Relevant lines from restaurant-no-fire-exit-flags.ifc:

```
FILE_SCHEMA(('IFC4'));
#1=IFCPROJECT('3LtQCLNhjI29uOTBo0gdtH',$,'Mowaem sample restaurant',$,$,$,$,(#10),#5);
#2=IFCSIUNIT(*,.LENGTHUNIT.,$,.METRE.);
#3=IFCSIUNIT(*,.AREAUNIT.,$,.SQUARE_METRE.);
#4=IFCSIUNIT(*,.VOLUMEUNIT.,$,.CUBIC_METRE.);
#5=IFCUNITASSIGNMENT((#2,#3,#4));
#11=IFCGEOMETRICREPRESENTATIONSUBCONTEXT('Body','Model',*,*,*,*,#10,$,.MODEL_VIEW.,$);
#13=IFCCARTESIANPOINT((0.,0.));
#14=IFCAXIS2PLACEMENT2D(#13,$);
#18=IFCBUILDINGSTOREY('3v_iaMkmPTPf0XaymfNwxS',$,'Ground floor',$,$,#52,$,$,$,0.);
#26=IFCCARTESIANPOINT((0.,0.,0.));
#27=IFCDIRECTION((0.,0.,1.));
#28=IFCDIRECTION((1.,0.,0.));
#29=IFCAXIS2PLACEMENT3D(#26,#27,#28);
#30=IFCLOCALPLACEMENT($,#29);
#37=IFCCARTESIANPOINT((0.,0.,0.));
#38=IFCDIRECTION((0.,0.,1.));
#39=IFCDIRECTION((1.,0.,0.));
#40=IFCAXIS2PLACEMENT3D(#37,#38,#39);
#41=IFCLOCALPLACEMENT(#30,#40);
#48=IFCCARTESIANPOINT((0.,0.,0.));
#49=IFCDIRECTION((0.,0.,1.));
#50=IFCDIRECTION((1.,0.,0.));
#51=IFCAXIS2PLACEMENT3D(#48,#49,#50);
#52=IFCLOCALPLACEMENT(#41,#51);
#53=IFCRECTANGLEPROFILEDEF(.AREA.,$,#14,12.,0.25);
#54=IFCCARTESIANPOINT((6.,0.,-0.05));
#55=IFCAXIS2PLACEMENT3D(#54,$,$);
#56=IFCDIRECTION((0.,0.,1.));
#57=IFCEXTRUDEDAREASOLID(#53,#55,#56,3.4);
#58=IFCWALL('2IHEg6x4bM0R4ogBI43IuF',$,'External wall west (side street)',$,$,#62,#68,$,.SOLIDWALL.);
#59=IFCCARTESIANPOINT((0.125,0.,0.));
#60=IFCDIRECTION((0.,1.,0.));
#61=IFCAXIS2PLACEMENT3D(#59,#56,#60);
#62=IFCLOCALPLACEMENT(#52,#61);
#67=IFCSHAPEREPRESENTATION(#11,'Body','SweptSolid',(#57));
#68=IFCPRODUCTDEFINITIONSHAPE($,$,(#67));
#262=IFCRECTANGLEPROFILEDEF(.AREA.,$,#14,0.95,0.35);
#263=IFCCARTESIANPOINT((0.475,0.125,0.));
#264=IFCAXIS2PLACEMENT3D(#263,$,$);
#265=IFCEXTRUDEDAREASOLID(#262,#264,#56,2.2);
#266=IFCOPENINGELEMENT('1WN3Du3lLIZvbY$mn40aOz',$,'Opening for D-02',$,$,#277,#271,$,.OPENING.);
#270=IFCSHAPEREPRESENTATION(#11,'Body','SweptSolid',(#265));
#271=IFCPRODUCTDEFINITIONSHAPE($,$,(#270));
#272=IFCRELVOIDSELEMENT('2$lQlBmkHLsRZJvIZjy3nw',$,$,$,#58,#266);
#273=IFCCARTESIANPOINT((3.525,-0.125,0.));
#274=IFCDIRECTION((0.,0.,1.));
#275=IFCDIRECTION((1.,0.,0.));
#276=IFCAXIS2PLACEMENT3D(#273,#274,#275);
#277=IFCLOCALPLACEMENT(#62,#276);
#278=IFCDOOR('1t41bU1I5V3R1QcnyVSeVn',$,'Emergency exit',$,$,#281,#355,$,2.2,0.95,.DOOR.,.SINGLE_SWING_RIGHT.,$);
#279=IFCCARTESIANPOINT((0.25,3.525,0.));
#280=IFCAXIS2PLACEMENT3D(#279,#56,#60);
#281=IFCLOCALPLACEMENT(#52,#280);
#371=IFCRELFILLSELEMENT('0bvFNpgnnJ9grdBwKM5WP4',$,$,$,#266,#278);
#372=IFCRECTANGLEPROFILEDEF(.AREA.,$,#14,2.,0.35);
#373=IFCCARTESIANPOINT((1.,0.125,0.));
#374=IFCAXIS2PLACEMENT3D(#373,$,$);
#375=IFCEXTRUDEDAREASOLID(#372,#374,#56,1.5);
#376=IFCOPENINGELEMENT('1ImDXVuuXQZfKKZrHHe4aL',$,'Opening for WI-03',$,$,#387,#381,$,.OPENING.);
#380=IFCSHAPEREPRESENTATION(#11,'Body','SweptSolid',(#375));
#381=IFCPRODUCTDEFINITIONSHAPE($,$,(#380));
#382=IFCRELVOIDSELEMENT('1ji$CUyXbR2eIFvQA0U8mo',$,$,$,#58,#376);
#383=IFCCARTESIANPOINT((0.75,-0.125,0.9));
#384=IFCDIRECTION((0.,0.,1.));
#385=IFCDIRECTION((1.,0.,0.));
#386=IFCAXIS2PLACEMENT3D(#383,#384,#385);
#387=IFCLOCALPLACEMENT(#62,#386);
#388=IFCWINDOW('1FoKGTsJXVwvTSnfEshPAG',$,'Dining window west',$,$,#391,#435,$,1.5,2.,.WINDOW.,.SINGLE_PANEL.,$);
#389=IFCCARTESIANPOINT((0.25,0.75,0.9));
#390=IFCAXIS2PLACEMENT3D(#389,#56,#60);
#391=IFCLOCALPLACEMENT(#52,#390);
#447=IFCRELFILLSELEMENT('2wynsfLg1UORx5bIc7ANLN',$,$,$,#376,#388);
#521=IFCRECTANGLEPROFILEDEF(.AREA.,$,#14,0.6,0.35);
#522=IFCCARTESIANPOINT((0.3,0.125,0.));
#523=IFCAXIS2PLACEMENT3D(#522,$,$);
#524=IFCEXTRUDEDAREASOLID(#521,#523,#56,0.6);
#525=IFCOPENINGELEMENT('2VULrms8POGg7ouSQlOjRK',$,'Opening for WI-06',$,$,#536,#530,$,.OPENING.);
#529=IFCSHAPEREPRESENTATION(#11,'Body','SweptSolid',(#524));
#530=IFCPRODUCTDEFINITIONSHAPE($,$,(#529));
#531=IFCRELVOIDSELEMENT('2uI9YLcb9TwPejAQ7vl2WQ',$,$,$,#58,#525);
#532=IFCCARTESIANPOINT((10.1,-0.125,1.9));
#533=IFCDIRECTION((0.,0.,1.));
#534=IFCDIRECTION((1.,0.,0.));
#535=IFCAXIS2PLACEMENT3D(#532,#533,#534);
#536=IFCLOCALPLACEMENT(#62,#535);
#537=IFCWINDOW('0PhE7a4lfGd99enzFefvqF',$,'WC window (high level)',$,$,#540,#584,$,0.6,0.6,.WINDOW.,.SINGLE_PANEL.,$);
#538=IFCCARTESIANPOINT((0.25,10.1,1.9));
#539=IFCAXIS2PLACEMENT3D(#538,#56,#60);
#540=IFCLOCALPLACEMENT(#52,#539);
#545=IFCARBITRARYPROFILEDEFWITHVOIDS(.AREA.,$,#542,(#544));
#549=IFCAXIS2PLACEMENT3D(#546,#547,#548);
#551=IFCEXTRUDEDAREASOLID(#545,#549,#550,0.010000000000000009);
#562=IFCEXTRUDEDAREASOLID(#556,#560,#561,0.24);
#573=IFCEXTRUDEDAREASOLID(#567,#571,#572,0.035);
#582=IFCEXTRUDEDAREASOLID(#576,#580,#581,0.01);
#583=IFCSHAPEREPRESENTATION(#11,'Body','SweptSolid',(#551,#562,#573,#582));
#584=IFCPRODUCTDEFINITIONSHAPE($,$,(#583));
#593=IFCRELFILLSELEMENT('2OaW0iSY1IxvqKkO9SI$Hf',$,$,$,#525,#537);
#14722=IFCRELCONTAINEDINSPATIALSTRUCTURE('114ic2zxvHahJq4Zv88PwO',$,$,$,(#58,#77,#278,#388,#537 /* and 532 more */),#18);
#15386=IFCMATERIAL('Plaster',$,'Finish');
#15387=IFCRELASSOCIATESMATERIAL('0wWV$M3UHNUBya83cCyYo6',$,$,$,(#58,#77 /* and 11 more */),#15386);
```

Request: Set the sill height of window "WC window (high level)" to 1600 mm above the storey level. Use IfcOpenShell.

```python
import numpy as np
import ifcopenshell
import ifcopenshell.api.geometry
import ifcopenshell.geom
import ifcopenshell.util.element
import ifcopenshell.util.placement
import ifcopenshell.util.shape
import ifcopenshell.util.unit

model = ifcopenshell.open("restaurant-no-fire-exit-flags.ifc")
unit_scale = ifcopenshell.util.unit.calculate_unit_scale(model)

window = model.by_id(537)
opening = window.FillsVoids[0].RelatingOpeningElement
storey = ifcopenshell.util.element.get_container(window, ifc_class="IfcBuildingStorey")
level = ifcopenshell.util.placement.get_local_placement(storey.ObjectPlacement)[2, 3]

# The opening's origin need not be at the sill, so measure its lowest point.
shape = ifcopenshell.geom.create_shape(ifcopenshell.geom.settings(), opening)
bottom = ifcopenshell.util.shape.get_shape_bottom_elevation(shape, shape.geometry) / unit_scale
dz = level + 1.6 / unit_scale - bottom

shift = np.array([0.0, 0.0, dz])
# The window is not placed relative to its opening, so move both.
for product in (opening, window):
    matrix = ifcopenshell.util.placement.get_local_placement(product.ObjectPlacement)
    matrix[:3, 3] += shift
    ifcopenshell.api.geometry.edit_object_placement(model, product=product, matrix=matrix, is_si=False)

print(f"moved by {dz * unit_scale:+.3f} m")

model.write("restaurant-no-fire-exit-flags_v2.ifc")
```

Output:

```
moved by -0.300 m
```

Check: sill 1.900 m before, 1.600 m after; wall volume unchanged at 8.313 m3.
